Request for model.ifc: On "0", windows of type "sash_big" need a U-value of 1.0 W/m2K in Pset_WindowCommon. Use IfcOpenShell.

First a look at what the model holds.

```python
import ifcopenshell
import ifcopenshell.util.element

model = ifcopenshell.open("model.ifc")
print(model.schema)
storey = next(s for s in model.by_type("IfcBuildingStorey") if s.Name == "0")
windows = [e for e in ifcopenshell.util.element.get_decomposition(storey) if e.is_a("IfcWindow")]
seen = {}
for e in windows:
    element_type = ifcopenshell.util.element.get_type(e)
    key = (element_type.Name if element_type != e and element_type else None, ifcopenshell.util.element.get_pset(e, "Pset_WindowCommon", "ThermalTransmittance"))
    seen[key] = seen.get(key, 0) + 1
for (name, value), count in sorted(seen.items(), key=str):
    print(count, "x", name, "|", value)
```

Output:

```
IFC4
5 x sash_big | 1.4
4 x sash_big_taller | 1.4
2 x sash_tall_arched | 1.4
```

```python
import ifcopenshell
import ifcopenshell.api.pset
import ifcopenshell.util.element

model = ifcopenshell.open("model.ifc")

storey = next(s for s in model.by_type("IfcBuildingStorey") if s.Name == "0")
windows = [e for e in ifcopenshell.util.element.get_decomposition(storey) if e.is_a("IfcWindow")]

count = 0
for e in windows:
    element_type = ifcopenshell.util.element.get_type(e)
    if element_type in (None, e) or element_type.Name != "sash_big":
        continue
    # add_pset returns the element's existing set when there is one.
    pset = ifcopenshell.api.pset.add_pset(model, product=e, name="Pset_WindowCommon")
    ifcopenshell.api.pset.edit_pset(model, pset=pset, properties={"ThermalTransmittance": 1.0})
    count += 1

print(count, "windows updated")

model.write("model_updated.ifc")
```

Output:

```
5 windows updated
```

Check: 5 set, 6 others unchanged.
